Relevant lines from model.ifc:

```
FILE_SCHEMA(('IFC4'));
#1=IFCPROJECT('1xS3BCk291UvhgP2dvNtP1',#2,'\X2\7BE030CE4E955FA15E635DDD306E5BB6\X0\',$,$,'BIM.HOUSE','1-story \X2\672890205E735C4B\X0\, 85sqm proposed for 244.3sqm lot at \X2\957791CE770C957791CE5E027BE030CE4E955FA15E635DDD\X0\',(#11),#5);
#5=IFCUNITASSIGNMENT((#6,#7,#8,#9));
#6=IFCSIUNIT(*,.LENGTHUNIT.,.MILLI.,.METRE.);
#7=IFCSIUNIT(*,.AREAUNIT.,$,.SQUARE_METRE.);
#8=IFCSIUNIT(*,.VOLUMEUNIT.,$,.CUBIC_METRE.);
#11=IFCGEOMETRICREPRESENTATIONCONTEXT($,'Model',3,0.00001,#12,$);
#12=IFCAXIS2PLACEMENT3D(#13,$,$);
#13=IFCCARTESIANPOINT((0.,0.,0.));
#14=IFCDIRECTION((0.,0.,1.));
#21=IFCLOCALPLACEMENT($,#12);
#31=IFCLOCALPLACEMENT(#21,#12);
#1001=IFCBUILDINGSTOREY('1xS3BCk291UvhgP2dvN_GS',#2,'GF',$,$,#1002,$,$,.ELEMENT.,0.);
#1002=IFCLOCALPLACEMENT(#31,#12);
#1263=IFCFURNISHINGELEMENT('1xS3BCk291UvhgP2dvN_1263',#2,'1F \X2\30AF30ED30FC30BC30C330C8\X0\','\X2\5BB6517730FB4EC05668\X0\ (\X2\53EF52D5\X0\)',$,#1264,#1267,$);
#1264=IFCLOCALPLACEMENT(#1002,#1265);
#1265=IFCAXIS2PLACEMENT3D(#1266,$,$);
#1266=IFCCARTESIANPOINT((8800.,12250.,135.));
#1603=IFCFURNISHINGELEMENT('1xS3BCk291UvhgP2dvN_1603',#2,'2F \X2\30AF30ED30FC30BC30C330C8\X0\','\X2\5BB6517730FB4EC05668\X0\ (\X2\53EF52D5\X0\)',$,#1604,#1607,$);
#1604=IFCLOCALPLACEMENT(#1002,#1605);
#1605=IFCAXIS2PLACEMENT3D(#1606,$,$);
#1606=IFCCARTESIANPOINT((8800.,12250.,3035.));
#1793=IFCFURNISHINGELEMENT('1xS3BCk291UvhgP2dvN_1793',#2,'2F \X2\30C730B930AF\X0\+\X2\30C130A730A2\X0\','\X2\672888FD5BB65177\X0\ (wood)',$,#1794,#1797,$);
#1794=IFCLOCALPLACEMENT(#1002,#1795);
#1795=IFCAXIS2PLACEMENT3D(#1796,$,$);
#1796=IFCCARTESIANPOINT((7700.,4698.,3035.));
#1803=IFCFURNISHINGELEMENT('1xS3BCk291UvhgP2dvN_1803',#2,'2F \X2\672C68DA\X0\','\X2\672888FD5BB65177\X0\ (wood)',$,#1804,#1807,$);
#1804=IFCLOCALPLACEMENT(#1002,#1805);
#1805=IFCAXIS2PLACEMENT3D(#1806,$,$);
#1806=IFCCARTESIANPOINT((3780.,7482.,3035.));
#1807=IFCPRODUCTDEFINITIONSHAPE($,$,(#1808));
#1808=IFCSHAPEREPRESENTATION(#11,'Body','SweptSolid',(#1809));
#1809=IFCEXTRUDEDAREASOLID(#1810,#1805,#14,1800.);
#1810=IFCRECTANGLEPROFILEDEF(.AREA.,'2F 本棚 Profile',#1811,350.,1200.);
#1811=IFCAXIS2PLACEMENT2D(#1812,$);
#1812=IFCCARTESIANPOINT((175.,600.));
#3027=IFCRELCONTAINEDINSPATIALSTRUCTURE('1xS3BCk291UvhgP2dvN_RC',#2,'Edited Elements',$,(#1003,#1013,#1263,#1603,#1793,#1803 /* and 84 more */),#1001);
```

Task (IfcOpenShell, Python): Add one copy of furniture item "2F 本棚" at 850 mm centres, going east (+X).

```python
import numpy as np
import ifcopenshell
import ifcopenshell.api.geometry
import ifcopenshell.api.root
import ifcopenshell.util.element
import ifcopenshell.util.placement

model = ifcopenshell.open("model.ifc")


def reuse_history(source, copy):
    """copy_class also copies each property set's owner history, people and application; keep the originals."""
    for rel in copy.IsDefinedBy:
        if rel.is_a("IfcRelDefinesByProperties") and (history := rel.RelatingPropertyDefinition.OwnerHistory):
            rel.RelatingPropertyDefinition.OwnerHistory = source.OwnerHistory
            ifcopenshell.util.element.remove_deep2(model, history)


source = model.by_id(1803)
base = ifcopenshell.util.placement.get_local_placement(source.ObjectPlacement)
step = np.array([1.0, 0.0, 0.0]) * 850.0

for i in range(1, 2):
    copy = ifcopenshell.api.root.copy_class(model, product=source)
    copy.Representation = ifcopenshell.util.element.copy_deep(
        model, source.Representation, exclude=["IfcGeometricRepresentationContext", "IfcRepresentationMap"]
    )
    reuse_history(source, copy)
    matrix = base.copy()
    matrix[:3, 3] += i * step
    print("added at", matrix[:3, 3].round(3) + 0.0)
    ifcopenshell.api.geometry.edit_object_placement(model, product=copy, matrix=matrix, is_si=False)

model.write("model_v2.ifc")
```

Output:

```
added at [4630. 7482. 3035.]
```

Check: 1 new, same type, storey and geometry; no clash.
